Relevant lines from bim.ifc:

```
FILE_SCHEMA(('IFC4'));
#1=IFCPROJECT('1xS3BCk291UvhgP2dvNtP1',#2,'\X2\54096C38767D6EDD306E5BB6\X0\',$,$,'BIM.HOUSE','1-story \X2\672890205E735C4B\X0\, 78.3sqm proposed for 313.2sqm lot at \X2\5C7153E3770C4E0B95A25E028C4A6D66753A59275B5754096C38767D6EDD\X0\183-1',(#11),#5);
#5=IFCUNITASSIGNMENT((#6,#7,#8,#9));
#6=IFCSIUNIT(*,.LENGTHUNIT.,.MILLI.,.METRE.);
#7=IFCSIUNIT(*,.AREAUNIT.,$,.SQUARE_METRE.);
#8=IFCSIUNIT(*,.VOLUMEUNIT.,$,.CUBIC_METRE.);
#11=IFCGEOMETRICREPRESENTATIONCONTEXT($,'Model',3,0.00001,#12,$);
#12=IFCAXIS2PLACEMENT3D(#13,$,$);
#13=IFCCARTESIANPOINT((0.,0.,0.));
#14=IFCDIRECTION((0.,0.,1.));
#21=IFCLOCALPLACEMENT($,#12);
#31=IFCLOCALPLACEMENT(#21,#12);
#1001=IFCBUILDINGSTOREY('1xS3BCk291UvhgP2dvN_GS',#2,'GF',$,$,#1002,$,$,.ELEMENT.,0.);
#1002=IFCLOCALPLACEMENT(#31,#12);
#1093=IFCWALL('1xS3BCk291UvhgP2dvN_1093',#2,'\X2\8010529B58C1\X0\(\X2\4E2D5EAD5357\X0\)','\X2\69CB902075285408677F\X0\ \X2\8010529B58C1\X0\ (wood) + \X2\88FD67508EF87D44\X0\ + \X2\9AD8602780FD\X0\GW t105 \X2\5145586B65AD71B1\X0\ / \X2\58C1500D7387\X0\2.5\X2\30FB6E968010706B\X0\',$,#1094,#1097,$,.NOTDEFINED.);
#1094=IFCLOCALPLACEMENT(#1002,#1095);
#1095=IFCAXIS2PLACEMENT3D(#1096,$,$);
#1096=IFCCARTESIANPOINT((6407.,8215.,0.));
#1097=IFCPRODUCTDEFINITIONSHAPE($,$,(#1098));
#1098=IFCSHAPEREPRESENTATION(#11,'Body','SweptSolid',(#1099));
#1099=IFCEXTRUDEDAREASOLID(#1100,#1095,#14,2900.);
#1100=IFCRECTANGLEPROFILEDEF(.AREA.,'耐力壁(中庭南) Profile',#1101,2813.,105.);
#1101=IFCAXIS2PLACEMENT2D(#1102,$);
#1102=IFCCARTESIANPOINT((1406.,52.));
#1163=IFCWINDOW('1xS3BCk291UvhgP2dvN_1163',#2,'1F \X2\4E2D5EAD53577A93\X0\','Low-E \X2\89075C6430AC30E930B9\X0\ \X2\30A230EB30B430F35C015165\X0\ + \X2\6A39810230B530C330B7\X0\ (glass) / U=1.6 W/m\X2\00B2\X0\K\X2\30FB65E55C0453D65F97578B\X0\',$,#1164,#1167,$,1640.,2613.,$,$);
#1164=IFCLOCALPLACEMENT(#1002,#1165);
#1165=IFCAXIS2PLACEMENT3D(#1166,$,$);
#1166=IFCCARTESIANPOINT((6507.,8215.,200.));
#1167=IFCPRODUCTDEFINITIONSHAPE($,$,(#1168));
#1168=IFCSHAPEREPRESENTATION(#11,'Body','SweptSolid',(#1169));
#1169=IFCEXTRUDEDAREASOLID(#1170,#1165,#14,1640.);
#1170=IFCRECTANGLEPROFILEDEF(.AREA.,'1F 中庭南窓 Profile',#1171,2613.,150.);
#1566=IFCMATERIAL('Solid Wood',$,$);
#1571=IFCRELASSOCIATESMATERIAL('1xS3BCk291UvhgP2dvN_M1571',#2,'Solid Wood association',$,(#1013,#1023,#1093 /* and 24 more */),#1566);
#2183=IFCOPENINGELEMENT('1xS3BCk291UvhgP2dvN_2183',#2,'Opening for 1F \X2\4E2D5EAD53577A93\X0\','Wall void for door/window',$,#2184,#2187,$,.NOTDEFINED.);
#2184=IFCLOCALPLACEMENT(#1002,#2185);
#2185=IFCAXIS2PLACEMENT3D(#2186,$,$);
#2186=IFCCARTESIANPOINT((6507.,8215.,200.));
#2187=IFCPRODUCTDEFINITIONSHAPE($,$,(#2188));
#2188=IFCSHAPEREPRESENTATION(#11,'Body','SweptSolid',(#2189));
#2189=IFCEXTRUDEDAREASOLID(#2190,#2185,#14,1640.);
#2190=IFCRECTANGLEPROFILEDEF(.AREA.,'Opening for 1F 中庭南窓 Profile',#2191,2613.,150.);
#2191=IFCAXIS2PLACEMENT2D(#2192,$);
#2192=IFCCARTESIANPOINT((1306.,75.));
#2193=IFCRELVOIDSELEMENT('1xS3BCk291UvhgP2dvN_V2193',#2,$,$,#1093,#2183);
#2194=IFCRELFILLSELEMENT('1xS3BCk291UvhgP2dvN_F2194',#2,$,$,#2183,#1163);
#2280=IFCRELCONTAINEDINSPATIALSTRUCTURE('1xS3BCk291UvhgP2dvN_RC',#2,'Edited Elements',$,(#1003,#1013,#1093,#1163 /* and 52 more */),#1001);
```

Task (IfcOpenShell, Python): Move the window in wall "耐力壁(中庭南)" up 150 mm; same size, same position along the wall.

```python
import numpy as np
import ifcopenshell
import ifcopenshell.api.geometry
import ifcopenshell.util.placement
import ifcopenshell.util.unit

model = ifcopenshell.open("bim.ifc")
unit_scale = ifcopenshell.util.unit.calculate_unit_scale(model)

window = model.by_guid("1xS3BCk291UvhgP2dvN_1163")
opening = window.FillsVoids[0].RelatingOpeningElement
dz = 0.15 / unit_scale

shift = np.array([0.0, 0.0, dz])
# The window is not placed relative to its opening, so move both.
for product in (opening, window):
    matrix = ifcopenshell.util.placement.get_local_placement(product.ObjectPlacement)
    matrix[:3, 3] += shift
    ifcopenshell.api.geometry.edit_object_placement(model, product=product, matrix=matrix, is_si=False)

print(f"moved by {dz * unit_scale:+.3f} m")

model.write("bim_v2.ifc")
```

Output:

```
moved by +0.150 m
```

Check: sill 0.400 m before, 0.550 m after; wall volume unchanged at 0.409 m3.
